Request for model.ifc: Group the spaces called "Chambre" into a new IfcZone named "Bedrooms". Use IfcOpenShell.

First a look at what the model holds.

```python
import ifcopenshell

model = ifcopenshell.open("model.ifc")
print(model.schema)
seen = {}
for space in model.by_type("IfcSpace"):
    seen[space.LongName] = seen.get(space.LongName, 0) + 1
for name, count in sorted(seen.items(), key=str):
    print(count, "x", name)
print("zones:", [z.Name for z in model.by_type("IfcZone")][:20])
```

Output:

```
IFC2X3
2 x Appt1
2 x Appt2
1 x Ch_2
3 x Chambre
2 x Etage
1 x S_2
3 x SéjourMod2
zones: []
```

```python
import ifcopenshell
import ifcopenshell.api.group
import ifcopenshell.api.root

model = ifcopenshell.open("model.ifc")

names = {"Chambre"}
spaces = [s for s in model.by_type("IfcSpace") if s.LongName in names]

zone = ifcopenshell.api.root.create_entity(model, ifc_class="IfcZone", name="Bedrooms")
ifcopenshell.api.group.assign_group(model, products=spaces, group=zone)
print(len(spaces), "spaces in", zone.Name)

model.write("model_edited.ifc")
```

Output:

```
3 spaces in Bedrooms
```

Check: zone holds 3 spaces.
